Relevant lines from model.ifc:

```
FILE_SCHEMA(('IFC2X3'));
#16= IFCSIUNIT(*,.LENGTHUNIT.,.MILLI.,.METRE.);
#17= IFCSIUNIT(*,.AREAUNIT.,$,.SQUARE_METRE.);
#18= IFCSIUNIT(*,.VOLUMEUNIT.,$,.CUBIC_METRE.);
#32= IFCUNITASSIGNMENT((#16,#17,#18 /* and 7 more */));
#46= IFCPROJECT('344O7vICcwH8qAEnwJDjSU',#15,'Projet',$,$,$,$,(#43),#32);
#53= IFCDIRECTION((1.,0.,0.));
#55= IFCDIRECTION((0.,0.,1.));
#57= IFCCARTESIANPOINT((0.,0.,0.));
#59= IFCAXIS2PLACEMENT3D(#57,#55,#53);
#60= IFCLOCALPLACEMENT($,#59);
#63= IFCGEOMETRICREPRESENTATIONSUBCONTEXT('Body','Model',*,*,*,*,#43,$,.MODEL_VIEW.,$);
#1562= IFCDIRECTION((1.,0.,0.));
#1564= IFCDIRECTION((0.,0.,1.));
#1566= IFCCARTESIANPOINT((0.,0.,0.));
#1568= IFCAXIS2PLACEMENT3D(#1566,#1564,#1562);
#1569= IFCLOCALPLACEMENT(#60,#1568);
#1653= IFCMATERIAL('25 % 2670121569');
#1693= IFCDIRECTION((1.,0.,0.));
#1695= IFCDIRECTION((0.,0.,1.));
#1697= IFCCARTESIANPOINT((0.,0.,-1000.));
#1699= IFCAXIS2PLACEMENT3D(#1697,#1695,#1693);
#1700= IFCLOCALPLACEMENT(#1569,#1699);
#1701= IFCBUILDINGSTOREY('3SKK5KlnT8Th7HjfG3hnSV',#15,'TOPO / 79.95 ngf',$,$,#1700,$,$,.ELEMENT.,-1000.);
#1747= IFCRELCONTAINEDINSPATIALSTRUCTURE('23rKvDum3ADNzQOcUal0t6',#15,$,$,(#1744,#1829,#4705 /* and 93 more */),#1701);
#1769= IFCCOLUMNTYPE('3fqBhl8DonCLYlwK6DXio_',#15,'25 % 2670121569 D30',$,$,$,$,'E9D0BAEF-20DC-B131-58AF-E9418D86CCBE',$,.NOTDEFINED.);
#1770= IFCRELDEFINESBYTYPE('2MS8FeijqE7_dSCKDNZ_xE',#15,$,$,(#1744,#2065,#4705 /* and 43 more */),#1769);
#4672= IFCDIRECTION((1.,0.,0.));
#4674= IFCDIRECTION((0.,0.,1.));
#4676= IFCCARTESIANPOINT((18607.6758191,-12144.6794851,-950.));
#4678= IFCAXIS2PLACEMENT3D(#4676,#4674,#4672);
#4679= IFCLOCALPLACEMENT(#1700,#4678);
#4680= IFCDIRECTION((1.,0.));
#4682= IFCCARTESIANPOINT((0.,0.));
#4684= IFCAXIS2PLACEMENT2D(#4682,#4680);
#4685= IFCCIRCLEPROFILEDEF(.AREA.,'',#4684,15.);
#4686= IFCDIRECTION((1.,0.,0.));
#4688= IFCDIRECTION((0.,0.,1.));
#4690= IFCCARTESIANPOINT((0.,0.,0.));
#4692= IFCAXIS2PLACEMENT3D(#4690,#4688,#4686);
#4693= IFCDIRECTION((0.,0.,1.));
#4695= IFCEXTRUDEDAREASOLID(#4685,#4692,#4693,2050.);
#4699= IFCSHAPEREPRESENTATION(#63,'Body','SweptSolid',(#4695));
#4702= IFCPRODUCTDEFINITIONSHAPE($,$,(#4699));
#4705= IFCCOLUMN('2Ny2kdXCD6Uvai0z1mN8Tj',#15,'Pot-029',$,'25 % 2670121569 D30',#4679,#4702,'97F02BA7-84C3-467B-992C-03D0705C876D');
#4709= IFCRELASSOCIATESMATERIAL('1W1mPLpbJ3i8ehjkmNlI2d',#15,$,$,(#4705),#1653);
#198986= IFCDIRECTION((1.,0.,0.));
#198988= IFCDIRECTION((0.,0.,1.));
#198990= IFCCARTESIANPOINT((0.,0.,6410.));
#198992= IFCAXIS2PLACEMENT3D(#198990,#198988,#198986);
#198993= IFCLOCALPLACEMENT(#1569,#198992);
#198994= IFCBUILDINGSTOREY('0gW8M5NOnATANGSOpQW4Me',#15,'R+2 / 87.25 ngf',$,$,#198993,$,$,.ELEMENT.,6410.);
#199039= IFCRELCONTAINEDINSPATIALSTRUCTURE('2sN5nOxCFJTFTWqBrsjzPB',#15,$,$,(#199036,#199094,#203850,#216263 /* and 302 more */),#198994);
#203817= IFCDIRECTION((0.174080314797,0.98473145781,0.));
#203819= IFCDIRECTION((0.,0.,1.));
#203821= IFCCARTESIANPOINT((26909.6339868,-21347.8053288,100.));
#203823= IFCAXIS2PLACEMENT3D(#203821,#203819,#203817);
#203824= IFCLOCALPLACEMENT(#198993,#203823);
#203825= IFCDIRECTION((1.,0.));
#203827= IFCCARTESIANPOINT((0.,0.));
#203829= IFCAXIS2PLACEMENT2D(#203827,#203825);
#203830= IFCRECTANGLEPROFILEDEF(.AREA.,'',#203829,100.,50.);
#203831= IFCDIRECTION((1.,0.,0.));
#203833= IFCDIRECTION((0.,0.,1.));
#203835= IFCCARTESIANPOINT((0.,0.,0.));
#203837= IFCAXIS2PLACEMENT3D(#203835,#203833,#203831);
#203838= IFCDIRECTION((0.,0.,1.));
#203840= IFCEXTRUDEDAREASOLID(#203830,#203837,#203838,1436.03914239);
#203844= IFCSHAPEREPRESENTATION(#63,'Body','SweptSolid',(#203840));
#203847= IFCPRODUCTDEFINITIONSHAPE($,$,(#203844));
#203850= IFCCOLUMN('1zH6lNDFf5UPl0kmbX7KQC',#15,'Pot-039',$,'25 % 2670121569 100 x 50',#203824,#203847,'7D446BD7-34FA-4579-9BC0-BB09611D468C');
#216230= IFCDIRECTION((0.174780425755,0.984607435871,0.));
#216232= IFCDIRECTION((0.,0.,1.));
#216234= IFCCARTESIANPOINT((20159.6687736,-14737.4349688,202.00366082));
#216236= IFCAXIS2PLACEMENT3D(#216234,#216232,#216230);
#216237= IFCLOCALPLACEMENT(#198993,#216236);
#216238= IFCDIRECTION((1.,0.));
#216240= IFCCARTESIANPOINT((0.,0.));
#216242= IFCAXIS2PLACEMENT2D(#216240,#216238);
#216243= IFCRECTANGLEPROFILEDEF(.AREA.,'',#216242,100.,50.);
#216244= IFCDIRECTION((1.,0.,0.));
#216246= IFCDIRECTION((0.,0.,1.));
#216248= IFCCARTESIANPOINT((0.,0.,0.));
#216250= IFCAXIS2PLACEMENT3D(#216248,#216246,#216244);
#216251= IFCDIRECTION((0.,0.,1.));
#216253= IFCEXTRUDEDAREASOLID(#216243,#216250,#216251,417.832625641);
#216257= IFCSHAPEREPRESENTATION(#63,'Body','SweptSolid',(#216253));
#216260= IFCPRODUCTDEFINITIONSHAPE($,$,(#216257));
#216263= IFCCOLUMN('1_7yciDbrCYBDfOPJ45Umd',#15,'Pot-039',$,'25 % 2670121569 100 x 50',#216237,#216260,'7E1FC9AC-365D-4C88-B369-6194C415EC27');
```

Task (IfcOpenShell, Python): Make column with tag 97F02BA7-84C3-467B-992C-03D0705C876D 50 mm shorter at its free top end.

```python
import ifcopenshell
import ifcopenshell.util.representation
import ifcopenshell.util.unit

model = ifcopenshell.open("model.ifc")
unit_scale = ifcopenshell.util.unit.calculate_unit_scale(model)

member = model.by_id(4705)
change = -0.05 / unit_scale

# The extrusion runs towards the end named, so only its depth changes.
body = ifcopenshell.util.representation.get_representation(member, "Model", "Body")
solid = body.Items[0]
old_length = solid.Depth
solid.Depth += change

print(f"length {old_length:g} -> {solid.Depth:g}")

model.write("model_updated.ifc")
```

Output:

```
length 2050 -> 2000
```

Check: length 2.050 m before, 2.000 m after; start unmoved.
